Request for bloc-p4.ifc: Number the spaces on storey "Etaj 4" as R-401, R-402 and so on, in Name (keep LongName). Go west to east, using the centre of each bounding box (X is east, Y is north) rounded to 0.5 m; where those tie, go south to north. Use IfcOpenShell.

First a look at what the model holds.

```python
import ifcopenshell
import ifcopenshell.util.element
import ifcopenshell.util.placement

model = ifcopenshell.open("bloc-p4.ifc")
print(model.schema)
storey = next(s for s in model.by_type("IfcBuildingStorey") if s.Name == "Etaj 4")
spaces = [e for e in ifcopenshell.util.element.get_decomposition(storey) if e.is_a("IfcSpace")]
for e in sorted(spaces, key=lambda e: e.id()):
    origin = ifcopenshell.util.placement.get_local_placement(e.ObjectPlacement)[:3, 3]
    print(e.id(), e.Name, e.LongName, origin.round(2) + 0.0, sep=" | ")
```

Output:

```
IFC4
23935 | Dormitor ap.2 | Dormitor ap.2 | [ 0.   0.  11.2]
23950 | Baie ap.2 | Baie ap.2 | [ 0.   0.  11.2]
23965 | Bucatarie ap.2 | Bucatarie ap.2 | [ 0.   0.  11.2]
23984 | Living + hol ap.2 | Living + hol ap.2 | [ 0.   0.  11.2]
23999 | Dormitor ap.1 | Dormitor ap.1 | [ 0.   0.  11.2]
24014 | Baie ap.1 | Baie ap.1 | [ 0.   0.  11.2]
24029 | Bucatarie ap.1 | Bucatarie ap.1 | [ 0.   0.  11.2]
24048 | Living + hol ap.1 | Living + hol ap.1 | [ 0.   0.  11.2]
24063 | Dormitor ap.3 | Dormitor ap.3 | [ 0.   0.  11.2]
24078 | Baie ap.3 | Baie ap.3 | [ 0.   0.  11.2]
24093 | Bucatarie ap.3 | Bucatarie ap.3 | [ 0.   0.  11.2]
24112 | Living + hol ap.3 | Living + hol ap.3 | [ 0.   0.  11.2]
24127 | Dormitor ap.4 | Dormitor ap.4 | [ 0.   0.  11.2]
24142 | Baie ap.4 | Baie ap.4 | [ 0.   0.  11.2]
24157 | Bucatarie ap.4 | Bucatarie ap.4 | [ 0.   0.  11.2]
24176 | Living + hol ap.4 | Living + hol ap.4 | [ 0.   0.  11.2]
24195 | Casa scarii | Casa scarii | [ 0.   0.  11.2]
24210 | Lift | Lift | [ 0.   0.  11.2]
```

```python
import ifcopenshell
import ifcopenshell.geom
import ifcopenshell.util.element
import ifcopenshell.util.shape

model = ifcopenshell.open("bloc-p4.ifc")
settings = ifcopenshell.geom.settings()
settings.set("use-world-coords", True)


def centre(element):
    shape = ifcopenshell.geom.create_shape(settings, element)
    return ifcopenshell.util.shape.get_bbox_centroid(shape.geometry)


storey = next(s for s in model.by_type("IfcBuildingStorey") if s.Name == "Etaj 4")
spaces = [e for e in ifcopenshell.util.element.get_decomposition(storey) if e.is_a("IfcSpace")]

# Insertion points can sit at a corner or the storey origin, so sort by the geometry (in metres).
centres = {e: centre(e) for e in spaces}
spaces.sort(key=lambda e: (round(centres[e][0] / 0.5), centres[e][1]))

for i, e in enumerate(spaces, start=1):
    number = f"R-4{i:02d}"
    e.Name = number
    print(e.id(), number)

model.write("bloc-p4_edited.ifc")
```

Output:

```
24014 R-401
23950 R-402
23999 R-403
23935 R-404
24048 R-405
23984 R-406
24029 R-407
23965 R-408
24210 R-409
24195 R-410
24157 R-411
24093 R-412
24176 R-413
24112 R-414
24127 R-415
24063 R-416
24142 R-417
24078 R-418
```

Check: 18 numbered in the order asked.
